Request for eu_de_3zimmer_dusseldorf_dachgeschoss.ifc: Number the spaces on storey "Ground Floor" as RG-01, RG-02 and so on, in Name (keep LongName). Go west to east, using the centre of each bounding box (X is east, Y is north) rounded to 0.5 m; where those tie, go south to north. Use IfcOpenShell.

First a look at what the model holds.

```python
import ifcopenshell
import ifcopenshell.util.element
import ifcopenshell.util.placement

model = ifcopenshell.open("eu_de_3zimmer_dusseldorf_dachgeschoss.ifc")
print(model.schema)
storey = next(s for s in model.by_type("IfcBuildingStorey") if s.Name == "Ground Floor")
spaces = [e for e in ifcopenshell.util.element.get_decomposition(storey) if e.is_a("IfcSpace")]
for e in sorted(spaces, key=lambda e: e.id()):
    origin = ifcopenshell.util.placement.get_local_placement(e.ObjectPlacement)[:3, 3]
    print(e.id(), e.Name, e.LongName, origin.round(2) + 0.0, sep=" | ")
```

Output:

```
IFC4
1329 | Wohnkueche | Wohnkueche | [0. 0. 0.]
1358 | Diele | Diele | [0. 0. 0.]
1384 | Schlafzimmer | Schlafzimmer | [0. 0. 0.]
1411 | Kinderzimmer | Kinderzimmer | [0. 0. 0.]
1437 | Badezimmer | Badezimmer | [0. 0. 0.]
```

```python
import ifcopenshell
import ifcopenshell.geom
import ifcopenshell.util.element
import ifcopenshell.util.shape

model = ifcopenshell.open("eu_de_3zimmer_dusseldorf_dachgeschoss.ifc")
settings = ifcopenshell.geom.settings()
settings.set("use-world-coords", True)


def centre(element):
    shape = ifcopenshell.geom.create_shape(settings, element)
    return ifcopenshell.util.shape.get_bbox_centroid(shape.geometry)


storey = next(s for s in model.by_type("IfcBuildingStorey") if s.Name == "Ground Floor")
spaces = [e for e in ifcopenshell.util.element.get_decomposition(storey) if e.is_a("IfcSpace")]

# Insertion points can sit at a corner or the storey origin, so sort by the geometry (in metres).
centres = {e: centre(e) for e in spaces}
spaces.sort(key=lambda e: (round(centres[e][0] / 0.5), centres[e][1]))

for i, e in enumerate(spaces, start=1):
    number = f"RG-{i:02d}"
    e.Name = number
    print(e.id(), number)

model.write("eu_de_3zimmer_dusseldorf_dachgeschoss-out.ifc")
```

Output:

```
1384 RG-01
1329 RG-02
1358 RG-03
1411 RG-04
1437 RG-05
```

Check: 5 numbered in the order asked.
